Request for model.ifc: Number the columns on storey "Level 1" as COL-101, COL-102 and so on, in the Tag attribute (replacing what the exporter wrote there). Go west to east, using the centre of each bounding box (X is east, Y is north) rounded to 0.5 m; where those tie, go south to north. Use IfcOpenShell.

First a look at what the model holds.

```python
import ifcopenshell
import ifcopenshell.util.element
import ifcopenshell.util.placement

model = ifcopenshell.open("model.ifc")
print(model.schema)
storey = next(s for s in model.by_type("IfcBuildingStorey") if s.Name == "Level 1")
columns = [e for e in ifcopenshell.util.element.get_decomposition(storey) if e.is_a("IfcColumn")]
for e in sorted(columns, key=lambda e: e.id()):
    origin = ifcopenshell.util.placement.get_local_placement(e.ObjectPlacement)[:3, 3]
    print(e.id(), e.Tag, e.Name, origin.round(2) + 0.0, sep=" | ")
```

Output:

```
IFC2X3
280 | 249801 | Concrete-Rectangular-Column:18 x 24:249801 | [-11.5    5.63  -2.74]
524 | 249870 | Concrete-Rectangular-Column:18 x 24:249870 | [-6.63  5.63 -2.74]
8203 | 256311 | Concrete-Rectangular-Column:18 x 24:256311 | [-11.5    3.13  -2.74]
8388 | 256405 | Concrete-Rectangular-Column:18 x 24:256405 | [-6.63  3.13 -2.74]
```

```python
import ifcopenshell
import ifcopenshell.geom
import ifcopenshell.util.element
import ifcopenshell.util.shape

model = ifcopenshell.open("model.ifc")
settings = ifcopenshell.geom.settings()
settings.set("use-world-coords", True)


def centre(element):
    shape = ifcopenshell.geom.create_shape(settings, element)
    return ifcopenshell.util.shape.get_bbox_centroid(shape.geometry)


storey = next(s for s in model.by_type("IfcBuildingStorey") if s.Name == "Level 1")
columns = [e for e in ifcopenshell.util.element.get_decomposition(storey) if e.is_a("IfcColumn")]

# Insertion points can sit at a corner or the storey origin, so sort by the geometry (in metres).
centres = {e: centre(e) for e in columns}
columns.sort(key=lambda e: (round(centres[e][0] / 0.5), centres[e][1]))

for i, e in enumerate(columns, start=1):
    number = f"COL-1{i:02d}"
    e.Tag = number
    print(e.id(), number)

model.write("model_v2.ifc")
```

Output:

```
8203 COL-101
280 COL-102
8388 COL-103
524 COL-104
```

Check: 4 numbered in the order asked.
